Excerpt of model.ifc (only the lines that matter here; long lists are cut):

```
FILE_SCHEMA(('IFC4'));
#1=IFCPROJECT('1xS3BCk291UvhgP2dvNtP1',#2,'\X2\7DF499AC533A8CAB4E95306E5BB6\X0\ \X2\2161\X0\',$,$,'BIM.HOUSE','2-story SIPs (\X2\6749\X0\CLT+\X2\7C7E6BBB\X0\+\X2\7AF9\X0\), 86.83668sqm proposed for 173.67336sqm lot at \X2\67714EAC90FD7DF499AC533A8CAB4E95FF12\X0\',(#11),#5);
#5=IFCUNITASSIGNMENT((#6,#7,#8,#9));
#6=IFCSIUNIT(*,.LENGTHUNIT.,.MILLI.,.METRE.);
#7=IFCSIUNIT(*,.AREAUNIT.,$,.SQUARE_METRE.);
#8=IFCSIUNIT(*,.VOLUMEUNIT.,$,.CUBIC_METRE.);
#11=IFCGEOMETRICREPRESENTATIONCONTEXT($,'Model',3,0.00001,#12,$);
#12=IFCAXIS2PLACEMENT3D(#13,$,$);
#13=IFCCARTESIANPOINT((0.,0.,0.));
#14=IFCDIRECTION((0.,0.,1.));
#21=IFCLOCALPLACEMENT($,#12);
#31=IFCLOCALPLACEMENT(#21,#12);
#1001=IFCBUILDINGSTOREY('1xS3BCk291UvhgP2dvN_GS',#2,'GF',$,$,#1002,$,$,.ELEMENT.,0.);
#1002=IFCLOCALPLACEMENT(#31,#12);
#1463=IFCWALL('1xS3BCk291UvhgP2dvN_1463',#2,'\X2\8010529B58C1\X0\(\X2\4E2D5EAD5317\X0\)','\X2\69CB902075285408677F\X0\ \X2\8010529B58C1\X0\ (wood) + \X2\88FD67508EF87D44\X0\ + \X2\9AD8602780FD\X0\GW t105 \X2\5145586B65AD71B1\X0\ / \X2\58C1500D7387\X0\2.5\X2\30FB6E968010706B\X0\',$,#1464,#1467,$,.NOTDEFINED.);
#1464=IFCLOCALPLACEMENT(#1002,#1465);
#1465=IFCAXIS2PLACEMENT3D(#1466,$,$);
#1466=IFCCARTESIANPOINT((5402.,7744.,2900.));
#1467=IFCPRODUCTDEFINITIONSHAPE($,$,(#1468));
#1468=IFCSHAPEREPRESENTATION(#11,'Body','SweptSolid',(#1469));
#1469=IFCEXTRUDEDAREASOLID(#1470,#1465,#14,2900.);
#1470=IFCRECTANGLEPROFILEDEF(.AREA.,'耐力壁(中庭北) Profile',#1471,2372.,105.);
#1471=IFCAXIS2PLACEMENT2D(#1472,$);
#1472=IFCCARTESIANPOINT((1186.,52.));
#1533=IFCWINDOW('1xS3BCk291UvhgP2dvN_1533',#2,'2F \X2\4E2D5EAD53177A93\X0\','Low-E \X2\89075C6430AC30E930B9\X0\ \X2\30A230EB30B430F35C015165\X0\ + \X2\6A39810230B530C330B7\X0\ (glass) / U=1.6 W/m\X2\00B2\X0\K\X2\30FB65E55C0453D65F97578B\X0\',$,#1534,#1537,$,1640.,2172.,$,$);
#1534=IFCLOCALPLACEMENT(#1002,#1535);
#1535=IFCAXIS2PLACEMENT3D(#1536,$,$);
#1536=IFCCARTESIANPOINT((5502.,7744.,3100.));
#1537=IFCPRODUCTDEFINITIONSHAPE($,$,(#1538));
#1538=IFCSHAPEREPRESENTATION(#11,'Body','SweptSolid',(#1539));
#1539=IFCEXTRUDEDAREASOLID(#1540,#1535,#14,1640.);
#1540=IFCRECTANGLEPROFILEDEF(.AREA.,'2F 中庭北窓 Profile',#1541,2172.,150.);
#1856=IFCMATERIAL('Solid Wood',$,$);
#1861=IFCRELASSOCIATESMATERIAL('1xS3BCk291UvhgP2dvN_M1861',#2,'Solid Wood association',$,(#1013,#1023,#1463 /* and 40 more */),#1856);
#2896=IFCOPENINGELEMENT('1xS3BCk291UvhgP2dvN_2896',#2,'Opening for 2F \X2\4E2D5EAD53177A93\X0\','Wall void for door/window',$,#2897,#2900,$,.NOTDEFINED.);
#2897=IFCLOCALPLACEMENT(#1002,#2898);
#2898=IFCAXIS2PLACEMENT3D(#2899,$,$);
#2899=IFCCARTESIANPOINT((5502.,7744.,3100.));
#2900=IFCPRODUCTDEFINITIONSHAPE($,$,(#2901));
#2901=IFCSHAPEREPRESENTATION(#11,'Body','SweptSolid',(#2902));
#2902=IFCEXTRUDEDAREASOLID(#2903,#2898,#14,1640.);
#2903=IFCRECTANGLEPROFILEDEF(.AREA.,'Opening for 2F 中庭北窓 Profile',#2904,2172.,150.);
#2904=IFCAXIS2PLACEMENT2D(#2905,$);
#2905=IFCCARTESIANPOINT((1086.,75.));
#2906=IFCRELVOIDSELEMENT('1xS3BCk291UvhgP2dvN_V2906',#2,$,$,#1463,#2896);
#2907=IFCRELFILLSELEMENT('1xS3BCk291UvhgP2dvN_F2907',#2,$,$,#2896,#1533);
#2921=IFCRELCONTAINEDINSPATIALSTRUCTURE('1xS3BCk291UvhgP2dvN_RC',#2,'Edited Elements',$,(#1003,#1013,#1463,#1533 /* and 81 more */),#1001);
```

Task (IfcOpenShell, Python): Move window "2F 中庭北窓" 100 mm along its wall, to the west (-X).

```python
import ifcopenshell
import ifcopenshell.api.geometry
import ifcopenshell.util.placement

model = ifcopenshell.open("model.ifc")

window = model.by_guid("1xS3BCk291UvhgP2dvN_1533")
opening = window.FillsVoids[0].RelatingOpeningElement
wall = opening.VoidsElements[0].RelatingBuildingElement

wall_matrix = ifcopenshell.util.placement.get_local_placement(wall.ObjectPlacement)
shift = wall_matrix[:3, 0] * -100.0
before = ifcopenshell.util.placement.get_local_placement(window.ObjectPlacement)[:3, 3].copy()

# The window is not placed relative to its opening, so move both.
for product in (opening, window):
    matrix = ifcopenshell.util.placement.get_local_placement(product.ObjectPlacement)
    matrix[:3, 3] += shift
    ifcopenshell.api.geometry.edit_object_placement(model, product=product, matrix=matrix, is_si=False)

after = ifcopenshell.util.placement.get_local_placement(window.ObjectPlacement)[:3, 3]
print("window moved by", (after - before).round(3) + 0.0)

model.write("model_v2.ifc")
```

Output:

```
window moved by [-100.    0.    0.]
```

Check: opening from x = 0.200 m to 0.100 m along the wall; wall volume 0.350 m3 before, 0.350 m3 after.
